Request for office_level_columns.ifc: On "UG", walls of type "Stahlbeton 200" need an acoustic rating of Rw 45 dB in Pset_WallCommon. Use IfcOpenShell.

First a look at what the model holds.

```python
import ifcopenshell
import ifcopenshell.util.element

model = ifcopenshell.open("office_level_columns.ifc")
print(model.schema)
storey = next(s for s in model.by_type("IfcBuildingStorey") if s.Name == "UG")
walls = [e for e in ifcopenshell.util.element.get_decomposition(storey) if e.is_a("IfcWall")]
seen = {}
for e in walls:
    element_type = ifcopenshell.util.element.get_type(e)
    key = (element_type.Name if element_type != e and element_type else None, ifcopenshell.util.element.get_pset(e, "Pset_WallCommon", "AcousticRating"))
    seen[key] = seen.get(key, 0) + 1
for (name, value), count in sorted(seen.items(), key=str):
    print(count, "x", name, "|", value)
```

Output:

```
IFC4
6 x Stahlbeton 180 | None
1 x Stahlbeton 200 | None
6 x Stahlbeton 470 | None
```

```python
import ifcopenshell
import ifcopenshell.api.pset
import ifcopenshell.util.element

model = ifcopenshell.open("office_level_columns.ifc")

storey = next(s for s in model.by_type("IfcBuildingStorey") if s.Name == "UG")
walls = [e for e in ifcopenshell.util.element.get_decomposition(storey) if e.is_a("IfcWall")]

count = 0
for e in walls:
    element_type = ifcopenshell.util.element.get_type(e)
    if element_type in (None, e) or element_type.Name != "Stahlbeton 200":
        continue
    # add_pset returns the element's existing set when there is one.
    pset = ifcopenshell.api.pset.add_pset(model, product=e, name="Pset_WallCommon")
    ifcopenshell.api.pset.edit_pset(model, pset=pset, properties={"AcousticRating": "Rw 45 dB"})
    count += 1

print(count, "walls updated")

model.write("office_level_columns-out.ifc")
```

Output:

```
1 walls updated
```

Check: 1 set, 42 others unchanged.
